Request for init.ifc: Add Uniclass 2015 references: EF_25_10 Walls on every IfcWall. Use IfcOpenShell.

First a look at what the model holds.

```python
import ifcopenshell

model = ifcopenshell.open("init.ifc")
print(model.schema)
print("classifications:", [c.Name for c in model.by_type("IfcClassification")])
for ifc_class in ("IfcDoor", "IfcRoof", "IfcStair", "IfcWall", "IfcWindow"):
    print(ifc_class, len(model.by_type(ifc_class)))
```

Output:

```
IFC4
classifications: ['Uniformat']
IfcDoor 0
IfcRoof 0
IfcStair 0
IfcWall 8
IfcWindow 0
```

```python
import ifcopenshell
import ifcopenshell.api.classification

model = ifcopenshell.open("init.ifc")

system = ifcopenshell.api.classification.add_classification(model, classification="Uniclass 2015")

codes = {
    "IfcWall": ("EF_25_10", "Walls"),
}
for ifc_class, (code, name) in codes.items():
    products = model.by_type(ifc_class)
    ifcopenshell.api.classification.add_reference(
        model, products=products, classification=system, identification=code, name=name
    )
    print(code, len(products))

model.write("init-out.ifc")
```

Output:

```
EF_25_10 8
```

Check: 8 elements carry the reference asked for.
